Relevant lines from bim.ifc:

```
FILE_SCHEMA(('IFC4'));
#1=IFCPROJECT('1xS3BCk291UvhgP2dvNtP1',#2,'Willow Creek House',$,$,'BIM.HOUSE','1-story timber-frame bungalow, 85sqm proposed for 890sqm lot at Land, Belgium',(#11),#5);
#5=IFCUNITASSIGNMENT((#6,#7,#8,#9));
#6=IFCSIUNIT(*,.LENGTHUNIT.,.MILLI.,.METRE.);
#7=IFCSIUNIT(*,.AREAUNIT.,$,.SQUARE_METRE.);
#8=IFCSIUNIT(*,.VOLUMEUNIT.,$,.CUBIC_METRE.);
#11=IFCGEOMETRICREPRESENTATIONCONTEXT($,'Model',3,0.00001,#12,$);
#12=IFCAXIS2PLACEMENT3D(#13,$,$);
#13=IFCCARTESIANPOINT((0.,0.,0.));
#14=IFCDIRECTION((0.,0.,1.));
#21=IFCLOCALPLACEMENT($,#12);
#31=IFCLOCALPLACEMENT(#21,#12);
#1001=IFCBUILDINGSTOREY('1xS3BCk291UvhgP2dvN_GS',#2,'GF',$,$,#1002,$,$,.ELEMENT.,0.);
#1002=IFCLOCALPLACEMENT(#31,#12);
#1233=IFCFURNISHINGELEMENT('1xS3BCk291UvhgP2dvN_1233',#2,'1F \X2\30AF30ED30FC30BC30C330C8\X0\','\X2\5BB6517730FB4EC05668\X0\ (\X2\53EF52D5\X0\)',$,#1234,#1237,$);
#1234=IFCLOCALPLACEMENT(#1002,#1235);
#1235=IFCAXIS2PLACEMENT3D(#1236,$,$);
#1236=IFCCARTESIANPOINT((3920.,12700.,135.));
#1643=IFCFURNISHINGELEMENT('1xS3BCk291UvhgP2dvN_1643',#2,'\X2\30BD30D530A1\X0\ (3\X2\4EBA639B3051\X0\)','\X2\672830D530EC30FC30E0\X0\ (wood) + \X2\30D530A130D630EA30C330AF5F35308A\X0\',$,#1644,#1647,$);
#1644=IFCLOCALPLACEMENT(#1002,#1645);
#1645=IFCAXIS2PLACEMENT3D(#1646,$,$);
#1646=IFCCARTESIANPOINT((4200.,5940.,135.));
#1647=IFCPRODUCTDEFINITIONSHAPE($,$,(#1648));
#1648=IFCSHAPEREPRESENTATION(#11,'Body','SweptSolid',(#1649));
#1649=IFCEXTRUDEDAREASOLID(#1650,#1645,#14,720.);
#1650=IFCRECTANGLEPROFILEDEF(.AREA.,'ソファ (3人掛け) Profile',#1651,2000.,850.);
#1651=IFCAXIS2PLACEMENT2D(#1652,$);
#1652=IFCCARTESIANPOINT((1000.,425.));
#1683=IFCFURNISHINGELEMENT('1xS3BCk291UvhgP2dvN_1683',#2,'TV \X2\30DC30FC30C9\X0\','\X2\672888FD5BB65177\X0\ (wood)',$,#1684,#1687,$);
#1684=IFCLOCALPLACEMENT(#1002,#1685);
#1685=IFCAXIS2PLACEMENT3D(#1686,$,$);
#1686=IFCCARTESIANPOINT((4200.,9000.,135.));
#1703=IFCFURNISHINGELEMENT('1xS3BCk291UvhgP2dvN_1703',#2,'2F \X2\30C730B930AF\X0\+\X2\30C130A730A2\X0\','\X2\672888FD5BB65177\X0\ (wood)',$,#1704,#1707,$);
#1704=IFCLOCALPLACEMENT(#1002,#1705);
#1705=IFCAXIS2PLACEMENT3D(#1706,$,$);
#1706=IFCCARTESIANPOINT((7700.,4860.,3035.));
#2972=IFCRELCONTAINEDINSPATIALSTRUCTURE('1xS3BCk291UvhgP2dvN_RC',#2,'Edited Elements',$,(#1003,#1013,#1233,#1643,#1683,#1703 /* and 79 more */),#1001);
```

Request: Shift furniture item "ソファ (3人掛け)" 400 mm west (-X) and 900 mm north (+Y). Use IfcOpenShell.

```python
import ifcopenshell
import ifcopenshell.api.geometry
import ifcopenshell.util.placement

model = ifcopenshell.open("bim.ifc")

item = model.by_guid("1xS3BCk291UvhgP2dvN_1643")
matrix = ifcopenshell.util.placement.get_local_placement(item.ObjectPlacement)
matrix[0, 3] -= 400.0
matrix[1, 3] += 900.0
ifcopenshell.api.geometry.edit_object_placement(model, product=item, matrix=matrix, is_si=False)

print(ifcopenshell.util.placement.get_local_placement(item.ObjectPlacement).round(3) + 0.0)

model.write("bim_updated.ifc")
```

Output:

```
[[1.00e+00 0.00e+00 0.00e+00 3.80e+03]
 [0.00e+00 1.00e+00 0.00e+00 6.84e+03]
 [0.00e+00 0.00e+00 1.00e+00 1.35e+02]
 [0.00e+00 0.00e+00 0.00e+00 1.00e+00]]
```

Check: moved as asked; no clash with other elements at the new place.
